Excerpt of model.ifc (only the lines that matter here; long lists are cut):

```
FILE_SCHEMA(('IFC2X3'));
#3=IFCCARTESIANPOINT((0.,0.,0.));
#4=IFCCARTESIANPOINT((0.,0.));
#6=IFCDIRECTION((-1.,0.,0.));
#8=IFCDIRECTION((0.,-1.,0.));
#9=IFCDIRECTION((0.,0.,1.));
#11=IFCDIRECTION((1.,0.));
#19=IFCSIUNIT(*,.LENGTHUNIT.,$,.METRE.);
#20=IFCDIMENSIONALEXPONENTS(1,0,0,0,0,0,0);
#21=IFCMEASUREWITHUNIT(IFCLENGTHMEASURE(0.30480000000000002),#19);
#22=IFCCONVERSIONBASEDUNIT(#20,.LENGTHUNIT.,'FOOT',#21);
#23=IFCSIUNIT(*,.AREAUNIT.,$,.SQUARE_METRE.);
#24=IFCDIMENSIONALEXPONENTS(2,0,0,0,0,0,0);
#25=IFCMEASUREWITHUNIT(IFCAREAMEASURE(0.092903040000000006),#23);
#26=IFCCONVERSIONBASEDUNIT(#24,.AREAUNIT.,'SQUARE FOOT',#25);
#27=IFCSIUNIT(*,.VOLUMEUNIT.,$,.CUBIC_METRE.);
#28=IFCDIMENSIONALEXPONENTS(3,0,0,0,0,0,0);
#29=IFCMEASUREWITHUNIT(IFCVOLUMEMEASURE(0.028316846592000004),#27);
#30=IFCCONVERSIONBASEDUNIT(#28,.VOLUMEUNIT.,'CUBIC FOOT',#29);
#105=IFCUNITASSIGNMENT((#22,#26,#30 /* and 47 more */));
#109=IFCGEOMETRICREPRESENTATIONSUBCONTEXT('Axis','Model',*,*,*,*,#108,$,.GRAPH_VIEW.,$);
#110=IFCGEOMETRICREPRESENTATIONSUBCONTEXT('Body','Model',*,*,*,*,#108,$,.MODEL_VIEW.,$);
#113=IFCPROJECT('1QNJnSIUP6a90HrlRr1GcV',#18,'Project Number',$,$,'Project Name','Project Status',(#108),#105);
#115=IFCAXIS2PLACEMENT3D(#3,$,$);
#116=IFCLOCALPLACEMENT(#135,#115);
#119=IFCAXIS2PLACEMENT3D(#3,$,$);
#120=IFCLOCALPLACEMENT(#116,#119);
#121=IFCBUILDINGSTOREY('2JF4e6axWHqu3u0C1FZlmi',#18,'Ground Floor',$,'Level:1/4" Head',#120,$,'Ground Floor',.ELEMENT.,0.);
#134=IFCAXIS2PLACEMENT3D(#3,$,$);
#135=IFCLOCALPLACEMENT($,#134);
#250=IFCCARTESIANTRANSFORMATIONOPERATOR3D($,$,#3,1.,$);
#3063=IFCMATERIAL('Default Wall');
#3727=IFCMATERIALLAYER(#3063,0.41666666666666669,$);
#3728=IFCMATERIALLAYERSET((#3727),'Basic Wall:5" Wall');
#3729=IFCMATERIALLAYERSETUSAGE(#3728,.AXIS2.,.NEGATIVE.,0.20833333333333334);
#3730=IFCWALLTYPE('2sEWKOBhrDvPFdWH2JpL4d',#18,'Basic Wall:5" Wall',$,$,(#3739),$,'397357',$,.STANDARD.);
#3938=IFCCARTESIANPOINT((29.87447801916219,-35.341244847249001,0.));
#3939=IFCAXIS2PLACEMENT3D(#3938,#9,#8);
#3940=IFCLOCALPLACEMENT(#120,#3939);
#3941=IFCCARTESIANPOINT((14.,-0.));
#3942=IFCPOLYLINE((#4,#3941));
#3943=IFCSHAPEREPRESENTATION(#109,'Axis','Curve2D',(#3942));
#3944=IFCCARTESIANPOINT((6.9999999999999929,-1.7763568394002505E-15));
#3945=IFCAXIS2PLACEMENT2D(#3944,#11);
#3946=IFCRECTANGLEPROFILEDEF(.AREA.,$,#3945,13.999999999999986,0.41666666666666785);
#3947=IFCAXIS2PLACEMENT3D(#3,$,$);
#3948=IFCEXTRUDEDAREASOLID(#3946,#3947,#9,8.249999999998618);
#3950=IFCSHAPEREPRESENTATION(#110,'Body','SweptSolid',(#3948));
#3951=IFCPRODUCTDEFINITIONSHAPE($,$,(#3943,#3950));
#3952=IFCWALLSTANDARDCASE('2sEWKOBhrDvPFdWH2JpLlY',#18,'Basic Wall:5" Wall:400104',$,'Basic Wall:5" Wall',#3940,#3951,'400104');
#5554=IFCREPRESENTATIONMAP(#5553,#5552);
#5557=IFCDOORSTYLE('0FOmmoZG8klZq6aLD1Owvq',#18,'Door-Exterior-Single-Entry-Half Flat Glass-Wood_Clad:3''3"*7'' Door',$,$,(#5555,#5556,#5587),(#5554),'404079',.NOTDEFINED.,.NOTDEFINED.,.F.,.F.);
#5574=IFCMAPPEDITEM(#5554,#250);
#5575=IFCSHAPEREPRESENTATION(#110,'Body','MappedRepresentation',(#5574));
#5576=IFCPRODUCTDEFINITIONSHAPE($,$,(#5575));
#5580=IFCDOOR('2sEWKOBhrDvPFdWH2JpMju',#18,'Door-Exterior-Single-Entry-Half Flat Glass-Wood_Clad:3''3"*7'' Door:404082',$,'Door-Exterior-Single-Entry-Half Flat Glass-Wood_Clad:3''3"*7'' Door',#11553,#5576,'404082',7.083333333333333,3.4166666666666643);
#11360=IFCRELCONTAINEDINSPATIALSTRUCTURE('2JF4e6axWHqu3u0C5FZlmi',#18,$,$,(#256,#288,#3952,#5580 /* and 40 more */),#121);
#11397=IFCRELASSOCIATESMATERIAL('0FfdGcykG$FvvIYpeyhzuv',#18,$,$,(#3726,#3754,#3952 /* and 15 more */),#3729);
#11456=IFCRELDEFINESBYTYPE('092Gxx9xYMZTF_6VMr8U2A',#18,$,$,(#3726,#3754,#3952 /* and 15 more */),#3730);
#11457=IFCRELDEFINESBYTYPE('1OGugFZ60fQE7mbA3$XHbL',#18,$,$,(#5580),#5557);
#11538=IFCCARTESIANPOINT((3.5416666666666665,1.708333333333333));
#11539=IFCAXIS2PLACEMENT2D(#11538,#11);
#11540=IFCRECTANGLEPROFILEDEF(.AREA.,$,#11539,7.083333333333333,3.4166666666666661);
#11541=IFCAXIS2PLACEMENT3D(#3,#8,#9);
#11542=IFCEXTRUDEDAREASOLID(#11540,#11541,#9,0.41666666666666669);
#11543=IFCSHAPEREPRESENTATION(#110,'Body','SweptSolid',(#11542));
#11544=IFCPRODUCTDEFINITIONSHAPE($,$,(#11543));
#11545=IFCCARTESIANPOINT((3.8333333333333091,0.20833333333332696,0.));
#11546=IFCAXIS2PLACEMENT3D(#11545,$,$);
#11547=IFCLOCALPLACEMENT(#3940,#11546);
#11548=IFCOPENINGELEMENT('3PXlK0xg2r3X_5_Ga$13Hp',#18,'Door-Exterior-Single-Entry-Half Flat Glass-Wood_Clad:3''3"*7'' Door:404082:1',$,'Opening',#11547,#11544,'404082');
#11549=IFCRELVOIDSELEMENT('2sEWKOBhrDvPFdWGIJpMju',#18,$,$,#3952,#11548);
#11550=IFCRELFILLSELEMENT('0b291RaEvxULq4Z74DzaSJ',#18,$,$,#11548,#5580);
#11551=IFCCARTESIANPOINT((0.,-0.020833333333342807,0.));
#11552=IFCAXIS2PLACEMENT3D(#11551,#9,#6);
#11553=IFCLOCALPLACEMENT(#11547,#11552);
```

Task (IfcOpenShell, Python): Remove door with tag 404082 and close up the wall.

```python
import ifcopenshell
import ifcopenshell.api.feature
import ifcopenshell.api.root
import ifcopenshell.geom
import ifcopenshell.util.shape

model = ifcopenshell.open("model.ifc")
settings = ifcopenshell.geom.settings()


def volume(element):
    """Net volume in cubic metres, openings subtracted."""
    shape = ifcopenshell.geom.create_shape(settings, element)
    return ifcopenshell.util.shape.get_volume(shape.geometry)


door = model.by_guid("2sEWKOBhrDvPFdWH2JpMju")
opening = door.FillsVoids[0].RelatingOpeningElement
wall = opening.VoidsElements[0].RelatingBuildingElement
before = volume(wall)

ifcopenshell.api.root.remove_product(model, product=door)
ifcopenshell.api.feature.remove_feature(model, feature=opening)

after = volume(wall)

print(f"wall volume {before:.3f} -> {after:.3f} m3")

model.write("model_rev.ifc")
```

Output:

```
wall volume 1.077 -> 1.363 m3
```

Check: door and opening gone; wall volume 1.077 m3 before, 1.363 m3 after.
